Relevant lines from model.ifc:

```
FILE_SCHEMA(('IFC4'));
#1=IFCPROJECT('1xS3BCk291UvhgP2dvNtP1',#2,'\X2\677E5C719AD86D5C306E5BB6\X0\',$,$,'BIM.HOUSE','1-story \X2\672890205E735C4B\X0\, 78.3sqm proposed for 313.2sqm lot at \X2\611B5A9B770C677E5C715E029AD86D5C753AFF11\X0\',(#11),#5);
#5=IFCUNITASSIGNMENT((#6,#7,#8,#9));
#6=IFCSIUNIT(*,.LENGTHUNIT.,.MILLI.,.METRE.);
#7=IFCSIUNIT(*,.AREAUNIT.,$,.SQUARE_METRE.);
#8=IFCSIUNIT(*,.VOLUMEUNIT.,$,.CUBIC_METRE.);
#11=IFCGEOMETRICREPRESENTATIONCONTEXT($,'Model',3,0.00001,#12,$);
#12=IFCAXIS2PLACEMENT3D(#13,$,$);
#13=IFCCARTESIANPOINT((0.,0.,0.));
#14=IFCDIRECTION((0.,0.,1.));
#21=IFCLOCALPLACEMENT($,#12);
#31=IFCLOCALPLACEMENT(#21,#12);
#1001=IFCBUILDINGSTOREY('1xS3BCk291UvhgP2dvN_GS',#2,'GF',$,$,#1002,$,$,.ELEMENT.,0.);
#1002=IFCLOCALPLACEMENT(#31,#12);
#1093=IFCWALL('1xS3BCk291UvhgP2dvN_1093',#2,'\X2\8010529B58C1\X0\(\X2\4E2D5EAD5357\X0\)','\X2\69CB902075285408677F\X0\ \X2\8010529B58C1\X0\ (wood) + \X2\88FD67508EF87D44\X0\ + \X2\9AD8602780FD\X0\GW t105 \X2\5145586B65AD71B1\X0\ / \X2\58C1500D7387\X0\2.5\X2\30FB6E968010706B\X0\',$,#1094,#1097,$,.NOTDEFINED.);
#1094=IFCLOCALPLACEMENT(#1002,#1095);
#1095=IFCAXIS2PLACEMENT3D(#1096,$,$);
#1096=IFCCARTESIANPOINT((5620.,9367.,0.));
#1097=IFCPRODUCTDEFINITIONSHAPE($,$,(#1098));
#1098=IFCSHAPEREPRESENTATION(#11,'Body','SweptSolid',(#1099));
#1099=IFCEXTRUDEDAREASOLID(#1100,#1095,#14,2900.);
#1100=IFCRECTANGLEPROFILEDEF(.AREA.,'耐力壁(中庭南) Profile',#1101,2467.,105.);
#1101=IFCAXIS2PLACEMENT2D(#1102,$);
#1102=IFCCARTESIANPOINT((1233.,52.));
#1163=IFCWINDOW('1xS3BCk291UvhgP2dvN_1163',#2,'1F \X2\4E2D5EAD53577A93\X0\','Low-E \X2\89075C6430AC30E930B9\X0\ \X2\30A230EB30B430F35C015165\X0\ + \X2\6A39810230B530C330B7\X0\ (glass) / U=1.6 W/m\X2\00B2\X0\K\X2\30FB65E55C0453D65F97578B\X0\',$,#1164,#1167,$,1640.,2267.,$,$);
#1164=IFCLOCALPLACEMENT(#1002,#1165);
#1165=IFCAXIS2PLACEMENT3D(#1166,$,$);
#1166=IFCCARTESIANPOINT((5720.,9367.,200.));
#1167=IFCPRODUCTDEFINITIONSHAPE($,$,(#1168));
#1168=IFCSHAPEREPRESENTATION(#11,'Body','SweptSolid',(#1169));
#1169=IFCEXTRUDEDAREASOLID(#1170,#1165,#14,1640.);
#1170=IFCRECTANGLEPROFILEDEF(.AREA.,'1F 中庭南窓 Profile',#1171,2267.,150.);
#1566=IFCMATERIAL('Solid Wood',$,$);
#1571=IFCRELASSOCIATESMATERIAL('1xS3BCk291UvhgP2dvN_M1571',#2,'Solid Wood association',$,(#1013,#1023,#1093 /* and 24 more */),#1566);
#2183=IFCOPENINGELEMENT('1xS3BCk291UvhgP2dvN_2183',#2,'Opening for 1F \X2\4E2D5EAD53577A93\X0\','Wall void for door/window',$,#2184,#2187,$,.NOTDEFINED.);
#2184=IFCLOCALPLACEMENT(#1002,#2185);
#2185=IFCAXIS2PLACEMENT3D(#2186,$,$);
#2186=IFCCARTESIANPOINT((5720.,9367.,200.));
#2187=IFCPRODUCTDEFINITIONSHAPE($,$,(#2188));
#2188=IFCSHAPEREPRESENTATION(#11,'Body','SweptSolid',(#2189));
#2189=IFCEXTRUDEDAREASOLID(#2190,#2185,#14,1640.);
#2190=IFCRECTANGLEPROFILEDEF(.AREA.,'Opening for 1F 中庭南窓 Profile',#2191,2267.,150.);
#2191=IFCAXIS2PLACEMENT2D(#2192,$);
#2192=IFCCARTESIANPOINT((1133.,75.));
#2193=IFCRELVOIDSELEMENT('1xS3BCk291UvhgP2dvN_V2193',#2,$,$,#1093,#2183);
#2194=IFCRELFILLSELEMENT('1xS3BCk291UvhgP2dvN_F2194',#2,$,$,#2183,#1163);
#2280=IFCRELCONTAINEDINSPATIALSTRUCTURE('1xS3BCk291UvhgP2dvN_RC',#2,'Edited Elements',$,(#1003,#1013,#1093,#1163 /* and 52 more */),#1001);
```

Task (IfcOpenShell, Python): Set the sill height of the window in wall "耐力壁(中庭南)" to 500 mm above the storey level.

```python
import numpy as np
import ifcopenshell
import ifcopenshell.api.geometry
import ifcopenshell.geom
import ifcopenshell.util.element
import ifcopenshell.util.placement
import ifcopenshell.util.shape
import ifcopenshell.util.unit

model = ifcopenshell.open("model.ifc")
unit_scale = ifcopenshell.util.unit.calculate_unit_scale(model)

window = model.by_guid("1xS3BCk291UvhgP2dvN_1163")
opening = window.FillsVoids[0].RelatingOpeningElement
storey = ifcopenshell.util.element.get_container(window, ifc_class="IfcBuildingStorey")
level = ifcopenshell.util.placement.get_local_placement(storey.ObjectPlacement)[2, 3]

# The opening's origin need not be at the sill, so measure its lowest point.
shape = ifcopenshell.geom.create_shape(ifcopenshell.geom.settings(), opening)
bottom = ifcopenshell.util.shape.get_shape_bottom_elevation(shape, shape.geometry) / unit_scale
dz = level + 500.0 - bottom

shift = np.array([0.0, 0.0, dz])
# The window is not placed relative to its opening, so move both.
for product in (opening, window):
    matrix = ifcopenshell.util.placement.get_local_placement(product.ObjectPlacement)
    matrix[:3, 3] += shift
    ifcopenshell.api.geometry.edit_object_placement(model, product=product, matrix=matrix, is_si=False)

print(f"moved by {dz * unit_scale:+.3f} m")

model.write("model_updated.ifc")
```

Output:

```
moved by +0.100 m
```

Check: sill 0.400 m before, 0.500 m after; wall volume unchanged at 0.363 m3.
